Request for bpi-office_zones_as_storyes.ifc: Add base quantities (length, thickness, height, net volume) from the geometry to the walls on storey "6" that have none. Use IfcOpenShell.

First a look at what the model holds.

```python
import ifcopenshell
import ifcopenshell.util.element
import ifcopenshell.util.unit

model = ifcopenshell.open("bpi-office_zones_as_storyes.ifc")
print(model.schema)
for unit_type in ("LENGTHUNIT", "AREAUNIT", "VOLUMEUNIT"):
    print(unit_type, ifcopenshell.util.unit.calculate_unit_scale(model, unit_type))
storey = next(s for s in model.by_type("IfcBuildingStorey") if s.Name == "6")
walls = [e for e in ifcopenshell.util.element.get_decomposition(storey) if e.is_a("IfcWall")]
for e in sorted(walls, key=lambda e: e.id()):
    print(e.id(), e.is_a(), e.Name, list(ifcopenshell.util.element.get_psets(e, qtos_only=True)), sep=" | ")
```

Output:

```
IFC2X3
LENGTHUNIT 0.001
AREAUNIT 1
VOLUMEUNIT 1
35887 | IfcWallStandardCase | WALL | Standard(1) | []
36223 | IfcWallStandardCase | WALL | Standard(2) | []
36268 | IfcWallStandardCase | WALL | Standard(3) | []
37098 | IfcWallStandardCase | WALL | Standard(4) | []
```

```python
import ifcopenshell
import ifcopenshell.api.pset
import ifcopenshell.geom
import ifcopenshell.util.element
import ifcopenshell.util.shape
import ifcopenshell.util.unit

model = ifcopenshell.open("bpi-office_zones_as_storyes.ifc")
unit_scale = ifcopenshell.util.unit.calculate_unit_scale(model)
volume_scale = ifcopenshell.util.unit.calculate_unit_scale(model, "VOLUMEUNIT")
settings = ifcopenshell.geom.settings()

storey = next(s for s in model.by_type("IfcBuildingStorey") if s.Name == "6")
walls = [e for e in ifcopenshell.util.element.get_decomposition(storey) if e.is_a("IfcWall")]

for e in sorted(walls, key=lambda e: e.id()):
    if ifcopenshell.util.element.get_psets(e, qtos_only=True, should_inherit=False):
        continue
    # Geometry comes back in metres, in the element's own axes.
    shape = ifcopenshell.geom.create_shape(settings, e)
    values = {
        "Length": ifcopenshell.util.shape.get_x(shape.geometry) / unit_scale,
        "Width": ifcopenshell.util.shape.get_y(shape.geometry) / unit_scale,
        "Height": ifcopenshell.util.shape.get_z(shape.geometry) / unit_scale,
        "NetVolume": ifcopenshell.util.shape.get_volume(shape.geometry) / volume_scale,
    }
    qto = ifcopenshell.api.pset.add_qto(model, product=e, name="BaseQuantities")
    ifcopenshell.api.pset.edit_qto(model, qto=qto, properties=values)
    print(e.id(), {k: round(v, 3) for k, v in values.items()})

model.write("bpi-office_zones_as_storyes_v2.ifc")
```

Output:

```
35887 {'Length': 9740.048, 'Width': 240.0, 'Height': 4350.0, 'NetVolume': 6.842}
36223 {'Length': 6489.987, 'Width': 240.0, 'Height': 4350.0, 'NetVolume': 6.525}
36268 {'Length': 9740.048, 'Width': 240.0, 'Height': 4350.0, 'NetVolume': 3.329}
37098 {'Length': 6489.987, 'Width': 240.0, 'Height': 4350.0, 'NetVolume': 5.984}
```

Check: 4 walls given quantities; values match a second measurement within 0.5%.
